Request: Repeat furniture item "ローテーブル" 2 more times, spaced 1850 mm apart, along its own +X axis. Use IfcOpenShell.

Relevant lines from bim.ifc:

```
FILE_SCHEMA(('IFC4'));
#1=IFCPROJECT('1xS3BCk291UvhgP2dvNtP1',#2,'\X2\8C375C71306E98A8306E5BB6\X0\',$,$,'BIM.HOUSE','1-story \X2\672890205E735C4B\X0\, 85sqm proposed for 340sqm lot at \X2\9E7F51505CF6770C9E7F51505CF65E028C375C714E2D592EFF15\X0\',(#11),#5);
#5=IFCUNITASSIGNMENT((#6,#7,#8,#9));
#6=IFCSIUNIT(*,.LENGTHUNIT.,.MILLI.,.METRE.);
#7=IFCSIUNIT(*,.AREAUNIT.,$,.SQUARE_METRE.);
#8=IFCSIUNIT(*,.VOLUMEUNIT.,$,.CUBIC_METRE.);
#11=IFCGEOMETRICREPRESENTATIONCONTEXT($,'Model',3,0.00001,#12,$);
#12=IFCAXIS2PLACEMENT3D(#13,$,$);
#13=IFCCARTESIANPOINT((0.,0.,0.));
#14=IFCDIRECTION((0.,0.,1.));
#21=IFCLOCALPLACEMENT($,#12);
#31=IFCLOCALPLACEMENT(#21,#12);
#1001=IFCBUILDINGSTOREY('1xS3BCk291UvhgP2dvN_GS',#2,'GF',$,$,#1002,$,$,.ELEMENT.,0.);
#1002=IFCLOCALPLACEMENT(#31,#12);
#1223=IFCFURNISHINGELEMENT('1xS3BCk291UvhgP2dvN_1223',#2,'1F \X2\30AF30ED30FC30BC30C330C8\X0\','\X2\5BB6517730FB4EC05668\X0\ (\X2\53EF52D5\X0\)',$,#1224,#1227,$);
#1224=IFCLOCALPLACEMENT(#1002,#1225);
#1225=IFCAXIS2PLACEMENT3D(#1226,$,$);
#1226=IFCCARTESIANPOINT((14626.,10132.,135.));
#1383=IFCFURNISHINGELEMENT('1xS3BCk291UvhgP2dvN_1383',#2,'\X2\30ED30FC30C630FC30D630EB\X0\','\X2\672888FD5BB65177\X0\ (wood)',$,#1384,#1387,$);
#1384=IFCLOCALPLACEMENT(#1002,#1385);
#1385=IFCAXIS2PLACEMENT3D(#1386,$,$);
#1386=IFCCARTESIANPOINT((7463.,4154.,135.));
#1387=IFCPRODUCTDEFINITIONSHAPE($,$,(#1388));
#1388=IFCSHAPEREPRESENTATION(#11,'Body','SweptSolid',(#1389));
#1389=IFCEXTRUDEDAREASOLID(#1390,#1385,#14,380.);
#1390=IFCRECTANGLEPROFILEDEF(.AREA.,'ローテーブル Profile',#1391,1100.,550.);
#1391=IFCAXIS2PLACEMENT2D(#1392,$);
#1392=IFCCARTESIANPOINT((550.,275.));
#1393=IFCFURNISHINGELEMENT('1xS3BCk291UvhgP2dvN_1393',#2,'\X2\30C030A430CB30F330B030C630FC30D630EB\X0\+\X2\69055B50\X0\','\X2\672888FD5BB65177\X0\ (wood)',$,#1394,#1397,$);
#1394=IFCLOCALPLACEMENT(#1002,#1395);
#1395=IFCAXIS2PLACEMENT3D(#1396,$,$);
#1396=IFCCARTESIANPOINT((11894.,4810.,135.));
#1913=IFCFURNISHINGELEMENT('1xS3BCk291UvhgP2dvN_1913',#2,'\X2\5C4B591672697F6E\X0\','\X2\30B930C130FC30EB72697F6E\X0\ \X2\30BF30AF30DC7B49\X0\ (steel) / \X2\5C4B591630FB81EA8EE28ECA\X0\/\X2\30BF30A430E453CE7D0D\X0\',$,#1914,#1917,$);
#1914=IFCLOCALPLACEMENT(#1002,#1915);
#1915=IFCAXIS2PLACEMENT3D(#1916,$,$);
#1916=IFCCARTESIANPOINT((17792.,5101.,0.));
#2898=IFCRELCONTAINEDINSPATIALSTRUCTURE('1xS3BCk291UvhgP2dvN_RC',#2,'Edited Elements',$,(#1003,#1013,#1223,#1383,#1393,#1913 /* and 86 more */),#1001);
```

```python
import ifcopenshell
import ifcopenshell.api.geometry
import ifcopenshell.api.root
import ifcopenshell.util.element
import ifcopenshell.util.placement

model = ifcopenshell.open("bim.ifc")


def reuse_history(source, copy):
    """copy_class also copies each property set's owner history, people and application; keep the originals."""
    for rel in copy.IsDefinedBy:
        if rel.is_a("IfcRelDefinesByProperties") and (history := rel.RelatingPropertyDefinition.OwnerHistory):
            rel.RelatingPropertyDefinition.OwnerHistory = source.OwnerHistory
            ifcopenshell.util.element.remove_deep2(model, history)


source = model.by_guid("1xS3BCk291UvhgP2dvN_1383")
base = ifcopenshell.util.placement.get_local_placement(source.ObjectPlacement)
step = base[:3, 0] * 1850.0

for i in range(1, 3):
    copy = ifcopenshell.api.root.copy_class(model, product=source)
    copy.Representation = ifcopenshell.util.element.copy_deep(
        model, source.Representation, exclude=["IfcGeometricRepresentationContext", "IfcRepresentationMap"]
    )
    reuse_history(source, copy)
    matrix = base.copy()
    matrix[:3, 3] += i * step
    print("added at", matrix[:3, 3].round(3) + 0.0)
    ifcopenshell.api.geometry.edit_object_placement(model, product=copy, matrix=matrix, is_si=False)

model.write("bim_edited.ifc")
```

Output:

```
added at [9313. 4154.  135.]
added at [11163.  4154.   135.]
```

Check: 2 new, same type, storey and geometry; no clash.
